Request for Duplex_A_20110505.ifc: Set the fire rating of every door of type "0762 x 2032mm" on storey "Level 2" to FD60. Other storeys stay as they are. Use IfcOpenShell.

First a look at what the model holds.

```python
import ifcopenshell
import ifcopenshell.util.element

model = ifcopenshell.open("Duplex_A_20110505.ifc")
print(model.schema)
storey = next(s for s in model.by_type("IfcBuildingStorey") if s.Name == "Level 2")
doors = [e for e in ifcopenshell.util.element.get_decomposition(storey) if e.is_a("IfcDoor")]
seen = {}
for e in doors:
    element_type = ifcopenshell.util.element.get_type(e)
    key = (element_type.Name if element_type != e and element_type else None, ifcopenshell.util.element.get_pset(e, "Pset_DoorCommon", "FireRating"))
    seen[key] = seen.get(key, 0) + 1
for (name, value), count in sorted(seen.items(), key=str):
    print(count, "x", name, "|", value)
```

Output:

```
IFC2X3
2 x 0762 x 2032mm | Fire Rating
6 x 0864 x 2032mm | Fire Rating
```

```python
import ifcopenshell
import ifcopenshell.api.pset
import ifcopenshell.util.element

model = ifcopenshell.open("Duplex_A_20110505.ifc")

storey = next(s for s in model.by_type("IfcBuildingStorey") if s.Name == "Level 2")
doors = [e for e in ifcopenshell.util.element.get_decomposition(storey) if e.is_a("IfcDoor")]

count = 0
for e in doors:
    element_type = ifcopenshell.util.element.get_type(e)
    if element_type in (None, e) or element_type.Name != "0762 x 2032mm":
        continue
    # add_pset returns the element's existing set when there is one.
    pset = ifcopenshell.api.pset.add_pset(model, product=e, name="Pset_DoorCommon")
    ifcopenshell.api.pset.edit_pset(model, pset=pset, properties={"FireRating": "FD60"})
    count += 1

print(count, "doors updated")

model.write("Duplex_A_20110505_v2.ifc")
```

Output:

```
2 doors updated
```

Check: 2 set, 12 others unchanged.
